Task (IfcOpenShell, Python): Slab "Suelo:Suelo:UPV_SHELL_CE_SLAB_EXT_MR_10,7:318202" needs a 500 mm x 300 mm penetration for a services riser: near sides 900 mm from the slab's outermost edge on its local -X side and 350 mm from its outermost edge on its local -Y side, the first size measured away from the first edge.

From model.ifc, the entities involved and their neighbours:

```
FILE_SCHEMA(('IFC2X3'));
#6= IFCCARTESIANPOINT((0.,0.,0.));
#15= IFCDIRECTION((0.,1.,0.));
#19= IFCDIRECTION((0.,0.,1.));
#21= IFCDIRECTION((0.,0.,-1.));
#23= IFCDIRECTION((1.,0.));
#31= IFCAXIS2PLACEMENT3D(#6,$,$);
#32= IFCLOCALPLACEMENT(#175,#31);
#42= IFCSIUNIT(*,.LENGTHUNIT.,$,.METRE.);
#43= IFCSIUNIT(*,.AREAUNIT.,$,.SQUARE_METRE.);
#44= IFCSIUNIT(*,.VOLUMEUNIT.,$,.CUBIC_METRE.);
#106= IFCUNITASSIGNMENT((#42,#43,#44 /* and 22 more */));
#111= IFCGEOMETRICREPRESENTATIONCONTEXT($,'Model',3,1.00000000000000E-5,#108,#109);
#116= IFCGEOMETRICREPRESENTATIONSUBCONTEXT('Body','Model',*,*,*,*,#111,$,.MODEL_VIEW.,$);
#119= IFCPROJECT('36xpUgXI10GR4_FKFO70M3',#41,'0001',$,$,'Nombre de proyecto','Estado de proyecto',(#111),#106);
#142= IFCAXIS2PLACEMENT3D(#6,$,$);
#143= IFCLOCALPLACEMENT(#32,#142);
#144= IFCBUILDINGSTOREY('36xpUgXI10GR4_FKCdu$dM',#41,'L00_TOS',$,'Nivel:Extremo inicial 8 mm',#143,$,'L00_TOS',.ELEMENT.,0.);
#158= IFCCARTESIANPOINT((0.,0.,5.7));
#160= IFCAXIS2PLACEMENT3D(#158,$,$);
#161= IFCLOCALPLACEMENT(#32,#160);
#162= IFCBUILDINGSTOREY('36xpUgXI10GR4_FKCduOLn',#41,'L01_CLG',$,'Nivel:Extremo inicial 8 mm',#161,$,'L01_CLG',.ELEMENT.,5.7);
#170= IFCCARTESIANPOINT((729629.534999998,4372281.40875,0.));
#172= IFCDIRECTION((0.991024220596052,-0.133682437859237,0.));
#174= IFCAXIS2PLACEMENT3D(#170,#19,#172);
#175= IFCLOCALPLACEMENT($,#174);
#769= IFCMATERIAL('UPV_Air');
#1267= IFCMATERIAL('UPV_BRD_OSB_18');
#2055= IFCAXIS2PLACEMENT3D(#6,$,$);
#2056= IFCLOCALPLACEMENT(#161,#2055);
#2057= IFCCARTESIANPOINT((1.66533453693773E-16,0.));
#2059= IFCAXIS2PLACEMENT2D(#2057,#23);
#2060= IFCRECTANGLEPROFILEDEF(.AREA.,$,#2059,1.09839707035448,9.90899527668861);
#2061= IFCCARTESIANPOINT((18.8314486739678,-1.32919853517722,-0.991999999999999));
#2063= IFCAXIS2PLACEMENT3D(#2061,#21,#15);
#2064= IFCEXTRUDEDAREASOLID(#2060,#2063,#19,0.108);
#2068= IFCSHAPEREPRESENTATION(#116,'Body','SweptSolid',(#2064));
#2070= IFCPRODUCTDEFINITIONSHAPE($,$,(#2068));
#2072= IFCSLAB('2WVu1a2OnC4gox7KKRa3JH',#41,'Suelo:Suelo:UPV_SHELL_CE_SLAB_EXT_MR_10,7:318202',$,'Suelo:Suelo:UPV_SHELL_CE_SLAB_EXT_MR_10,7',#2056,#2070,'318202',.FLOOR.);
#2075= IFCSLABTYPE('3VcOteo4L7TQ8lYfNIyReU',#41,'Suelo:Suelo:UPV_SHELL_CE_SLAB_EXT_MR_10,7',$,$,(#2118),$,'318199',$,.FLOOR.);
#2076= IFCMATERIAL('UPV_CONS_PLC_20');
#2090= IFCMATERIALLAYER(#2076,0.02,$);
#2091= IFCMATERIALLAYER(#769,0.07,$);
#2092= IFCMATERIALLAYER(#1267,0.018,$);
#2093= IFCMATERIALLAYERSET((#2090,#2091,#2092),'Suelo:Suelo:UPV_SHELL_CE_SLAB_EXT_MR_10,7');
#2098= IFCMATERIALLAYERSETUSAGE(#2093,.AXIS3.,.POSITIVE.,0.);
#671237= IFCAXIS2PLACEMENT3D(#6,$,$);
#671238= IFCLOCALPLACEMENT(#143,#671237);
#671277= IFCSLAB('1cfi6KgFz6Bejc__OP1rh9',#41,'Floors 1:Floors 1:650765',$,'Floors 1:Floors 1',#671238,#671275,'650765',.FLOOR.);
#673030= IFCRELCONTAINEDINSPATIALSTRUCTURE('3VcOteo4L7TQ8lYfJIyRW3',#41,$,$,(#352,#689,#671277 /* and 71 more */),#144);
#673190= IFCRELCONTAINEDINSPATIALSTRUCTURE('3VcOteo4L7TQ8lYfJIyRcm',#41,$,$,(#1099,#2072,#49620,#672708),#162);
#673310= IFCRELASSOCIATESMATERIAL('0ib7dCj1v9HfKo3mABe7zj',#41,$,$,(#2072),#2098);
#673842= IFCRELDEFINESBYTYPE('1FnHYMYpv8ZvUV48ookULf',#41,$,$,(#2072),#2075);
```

```python
import numpy as np
import ifcopenshell
import ifcopenshell.api.feature
import ifcopenshell.api.geometry
import ifcopenshell.api.root
import ifcopenshell.geom
import ifcopenshell.util.placement
import ifcopenshell.util.representation
import ifcopenshell.util.shape
import ifcopenshell.util.unit

model = ifcopenshell.open("model.ifc")
unit_scale = ifcopenshell.util.unit.calculate_unit_scale(model)
settings = ifcopenshell.geom.settings()


def volume(element):
    """Net volume in cubic metres, openings subtracted."""
    shape = ifcopenshell.geom.create_shape(settings, element)
    return ifcopenshell.util.shape.get_volume(shape.geometry)


slab = model.by_guid("2WVu1a2OnC4gox7KKRa3JH")
before = volume(slab)

# Extent in the slab's own axes, in metres. The edges named are its -X and -Y sides.
slab_shape = ifcopenshell.geom.create_shape(settings, slab)
vertices = ifcopenshell.util.shape.get_vertices(slab_shape.geometry)
x_min, y_min, bottom = vertices.min(axis=0)
top = vertices[:, 2].max()

opening = ifcopenshell.api.root.create_entity(model, ifc_class="IfcOpeningElement", name="Services riser opening")
context = ifcopenshell.util.representation.get_context(model, "Model", "Body", "MODEL_VIEW")
width, depth = 0.5, 0.3
outline = [(0.0, 0.0), (width, 0.0), (width, depth), (0.0, depth), (0.0, 0.0)]
# Overshoot both faces by 50 mm so the cut is clean.
shape = ifcopenshell.api.geometry.add_slab_representation(
    model, context=context, depth=top - bottom + 0.1, polyline=outline
)
ifcopenshell.api.geometry.assign_representation(model, product=opening, representation=shape)

matrix = ifcopenshell.util.placement.get_local_placement(slab.ObjectPlacement)
matrix[:, 3] = matrix @ np.append(np.array([x_min + 0.9, y_min + 0.35, bottom - 0.05]) / unit_scale, 1.0)
ifcopenshell.api.geometry.edit_object_placement(model, product=opening, matrix=matrix, is_si=False)
ifcopenshell.api.feature.add_feature(model, feature=opening, element=slab)

after = volume(slab)

print(f"slab volume {before:.3f} -> {after:.3f} m3")

model.write("model_edited.ifc")
```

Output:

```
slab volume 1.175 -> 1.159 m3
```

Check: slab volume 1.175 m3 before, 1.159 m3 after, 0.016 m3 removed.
